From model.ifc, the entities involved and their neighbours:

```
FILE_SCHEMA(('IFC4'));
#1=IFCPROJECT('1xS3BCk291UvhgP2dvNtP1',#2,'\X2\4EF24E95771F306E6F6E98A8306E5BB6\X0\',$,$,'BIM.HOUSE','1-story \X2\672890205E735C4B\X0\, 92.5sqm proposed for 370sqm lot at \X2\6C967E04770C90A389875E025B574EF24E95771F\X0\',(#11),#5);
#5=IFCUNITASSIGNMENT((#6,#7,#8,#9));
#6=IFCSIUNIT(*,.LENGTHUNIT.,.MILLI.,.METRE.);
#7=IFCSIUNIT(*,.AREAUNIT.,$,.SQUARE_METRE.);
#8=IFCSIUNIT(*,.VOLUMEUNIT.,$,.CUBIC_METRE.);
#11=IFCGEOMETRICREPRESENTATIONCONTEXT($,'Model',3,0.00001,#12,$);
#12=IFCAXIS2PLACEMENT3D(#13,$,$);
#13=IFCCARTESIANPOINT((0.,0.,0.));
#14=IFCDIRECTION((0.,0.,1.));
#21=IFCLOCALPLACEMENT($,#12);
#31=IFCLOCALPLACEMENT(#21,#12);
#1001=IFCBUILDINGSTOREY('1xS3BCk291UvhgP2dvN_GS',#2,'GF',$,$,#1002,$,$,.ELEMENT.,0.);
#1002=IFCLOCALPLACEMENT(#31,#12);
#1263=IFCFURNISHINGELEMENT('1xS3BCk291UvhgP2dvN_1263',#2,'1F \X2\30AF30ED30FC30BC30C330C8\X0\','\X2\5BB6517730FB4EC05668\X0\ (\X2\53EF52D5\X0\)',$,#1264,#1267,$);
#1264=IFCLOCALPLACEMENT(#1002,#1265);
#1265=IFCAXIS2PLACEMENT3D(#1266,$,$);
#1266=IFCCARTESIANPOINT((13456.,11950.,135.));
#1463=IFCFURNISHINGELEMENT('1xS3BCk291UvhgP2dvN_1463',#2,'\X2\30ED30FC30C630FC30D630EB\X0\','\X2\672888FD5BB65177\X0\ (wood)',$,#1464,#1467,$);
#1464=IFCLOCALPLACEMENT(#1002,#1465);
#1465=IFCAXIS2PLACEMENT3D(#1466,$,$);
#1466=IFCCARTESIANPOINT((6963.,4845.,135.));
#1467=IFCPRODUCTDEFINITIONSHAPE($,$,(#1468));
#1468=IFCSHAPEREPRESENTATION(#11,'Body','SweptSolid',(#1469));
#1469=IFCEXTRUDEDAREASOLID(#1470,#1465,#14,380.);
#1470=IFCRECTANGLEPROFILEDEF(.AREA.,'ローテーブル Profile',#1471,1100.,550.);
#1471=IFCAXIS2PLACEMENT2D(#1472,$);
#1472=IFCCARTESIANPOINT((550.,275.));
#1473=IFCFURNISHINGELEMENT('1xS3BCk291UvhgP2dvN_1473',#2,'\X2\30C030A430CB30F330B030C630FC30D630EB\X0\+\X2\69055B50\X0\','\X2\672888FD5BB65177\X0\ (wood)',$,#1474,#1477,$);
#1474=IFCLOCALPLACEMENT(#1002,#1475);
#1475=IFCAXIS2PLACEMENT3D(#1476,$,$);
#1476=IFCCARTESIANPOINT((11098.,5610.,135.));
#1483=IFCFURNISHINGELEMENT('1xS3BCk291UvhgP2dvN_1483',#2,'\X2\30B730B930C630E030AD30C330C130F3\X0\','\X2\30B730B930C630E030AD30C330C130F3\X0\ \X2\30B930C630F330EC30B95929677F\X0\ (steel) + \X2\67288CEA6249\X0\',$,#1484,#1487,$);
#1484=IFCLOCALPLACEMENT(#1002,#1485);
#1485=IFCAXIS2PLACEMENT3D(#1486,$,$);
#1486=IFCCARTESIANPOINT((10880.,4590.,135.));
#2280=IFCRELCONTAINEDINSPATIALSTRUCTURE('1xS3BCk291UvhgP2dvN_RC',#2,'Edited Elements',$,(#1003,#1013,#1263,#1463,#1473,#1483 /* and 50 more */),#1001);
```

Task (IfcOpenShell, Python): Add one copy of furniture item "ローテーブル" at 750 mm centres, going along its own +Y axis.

```python
import ifcopenshell
import ifcopenshell.api.geometry
import ifcopenshell.api.root
import ifcopenshell.util.element
import ifcopenshell.util.placement

model = ifcopenshell.open("model.ifc")


def reuse_history(source, copy):
    """copy_class also copies each property set's owner history, people and application; keep the originals."""
    for rel in copy.IsDefinedBy:
        if rel.is_a("IfcRelDefinesByProperties") and (history := rel.RelatingPropertyDefinition.OwnerHistory):
            rel.RelatingPropertyDefinition.OwnerHistory = source.OwnerHistory
            ifcopenshell.util.element.remove_deep2(model, history)


source = model.by_guid("1xS3BCk291UvhgP2dvN_1463")
base = ifcopenshell.util.placement.get_local_placement(source.ObjectPlacement)
step = base[:3, 1] * 750.0

for i in range(1, 2):
    copy = ifcopenshell.api.root.copy_class(model, product=source)
    copy.Representation = ifcopenshell.util.element.copy_deep(
        model, source.Representation, exclude=["IfcGeometricRepresentationContext", "IfcRepresentationMap"]
    )
    reuse_history(source, copy)
    matrix = base.copy()
    matrix[:3, 3] += i * step
    print("added at", matrix[:3, 3].round(3) + 0.0)
    ifcopenshell.api.geometry.edit_object_placement(model, product=copy, matrix=matrix, is_si=False)

model.write("model_v2.ifc")
```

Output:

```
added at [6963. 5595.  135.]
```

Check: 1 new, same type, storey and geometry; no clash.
